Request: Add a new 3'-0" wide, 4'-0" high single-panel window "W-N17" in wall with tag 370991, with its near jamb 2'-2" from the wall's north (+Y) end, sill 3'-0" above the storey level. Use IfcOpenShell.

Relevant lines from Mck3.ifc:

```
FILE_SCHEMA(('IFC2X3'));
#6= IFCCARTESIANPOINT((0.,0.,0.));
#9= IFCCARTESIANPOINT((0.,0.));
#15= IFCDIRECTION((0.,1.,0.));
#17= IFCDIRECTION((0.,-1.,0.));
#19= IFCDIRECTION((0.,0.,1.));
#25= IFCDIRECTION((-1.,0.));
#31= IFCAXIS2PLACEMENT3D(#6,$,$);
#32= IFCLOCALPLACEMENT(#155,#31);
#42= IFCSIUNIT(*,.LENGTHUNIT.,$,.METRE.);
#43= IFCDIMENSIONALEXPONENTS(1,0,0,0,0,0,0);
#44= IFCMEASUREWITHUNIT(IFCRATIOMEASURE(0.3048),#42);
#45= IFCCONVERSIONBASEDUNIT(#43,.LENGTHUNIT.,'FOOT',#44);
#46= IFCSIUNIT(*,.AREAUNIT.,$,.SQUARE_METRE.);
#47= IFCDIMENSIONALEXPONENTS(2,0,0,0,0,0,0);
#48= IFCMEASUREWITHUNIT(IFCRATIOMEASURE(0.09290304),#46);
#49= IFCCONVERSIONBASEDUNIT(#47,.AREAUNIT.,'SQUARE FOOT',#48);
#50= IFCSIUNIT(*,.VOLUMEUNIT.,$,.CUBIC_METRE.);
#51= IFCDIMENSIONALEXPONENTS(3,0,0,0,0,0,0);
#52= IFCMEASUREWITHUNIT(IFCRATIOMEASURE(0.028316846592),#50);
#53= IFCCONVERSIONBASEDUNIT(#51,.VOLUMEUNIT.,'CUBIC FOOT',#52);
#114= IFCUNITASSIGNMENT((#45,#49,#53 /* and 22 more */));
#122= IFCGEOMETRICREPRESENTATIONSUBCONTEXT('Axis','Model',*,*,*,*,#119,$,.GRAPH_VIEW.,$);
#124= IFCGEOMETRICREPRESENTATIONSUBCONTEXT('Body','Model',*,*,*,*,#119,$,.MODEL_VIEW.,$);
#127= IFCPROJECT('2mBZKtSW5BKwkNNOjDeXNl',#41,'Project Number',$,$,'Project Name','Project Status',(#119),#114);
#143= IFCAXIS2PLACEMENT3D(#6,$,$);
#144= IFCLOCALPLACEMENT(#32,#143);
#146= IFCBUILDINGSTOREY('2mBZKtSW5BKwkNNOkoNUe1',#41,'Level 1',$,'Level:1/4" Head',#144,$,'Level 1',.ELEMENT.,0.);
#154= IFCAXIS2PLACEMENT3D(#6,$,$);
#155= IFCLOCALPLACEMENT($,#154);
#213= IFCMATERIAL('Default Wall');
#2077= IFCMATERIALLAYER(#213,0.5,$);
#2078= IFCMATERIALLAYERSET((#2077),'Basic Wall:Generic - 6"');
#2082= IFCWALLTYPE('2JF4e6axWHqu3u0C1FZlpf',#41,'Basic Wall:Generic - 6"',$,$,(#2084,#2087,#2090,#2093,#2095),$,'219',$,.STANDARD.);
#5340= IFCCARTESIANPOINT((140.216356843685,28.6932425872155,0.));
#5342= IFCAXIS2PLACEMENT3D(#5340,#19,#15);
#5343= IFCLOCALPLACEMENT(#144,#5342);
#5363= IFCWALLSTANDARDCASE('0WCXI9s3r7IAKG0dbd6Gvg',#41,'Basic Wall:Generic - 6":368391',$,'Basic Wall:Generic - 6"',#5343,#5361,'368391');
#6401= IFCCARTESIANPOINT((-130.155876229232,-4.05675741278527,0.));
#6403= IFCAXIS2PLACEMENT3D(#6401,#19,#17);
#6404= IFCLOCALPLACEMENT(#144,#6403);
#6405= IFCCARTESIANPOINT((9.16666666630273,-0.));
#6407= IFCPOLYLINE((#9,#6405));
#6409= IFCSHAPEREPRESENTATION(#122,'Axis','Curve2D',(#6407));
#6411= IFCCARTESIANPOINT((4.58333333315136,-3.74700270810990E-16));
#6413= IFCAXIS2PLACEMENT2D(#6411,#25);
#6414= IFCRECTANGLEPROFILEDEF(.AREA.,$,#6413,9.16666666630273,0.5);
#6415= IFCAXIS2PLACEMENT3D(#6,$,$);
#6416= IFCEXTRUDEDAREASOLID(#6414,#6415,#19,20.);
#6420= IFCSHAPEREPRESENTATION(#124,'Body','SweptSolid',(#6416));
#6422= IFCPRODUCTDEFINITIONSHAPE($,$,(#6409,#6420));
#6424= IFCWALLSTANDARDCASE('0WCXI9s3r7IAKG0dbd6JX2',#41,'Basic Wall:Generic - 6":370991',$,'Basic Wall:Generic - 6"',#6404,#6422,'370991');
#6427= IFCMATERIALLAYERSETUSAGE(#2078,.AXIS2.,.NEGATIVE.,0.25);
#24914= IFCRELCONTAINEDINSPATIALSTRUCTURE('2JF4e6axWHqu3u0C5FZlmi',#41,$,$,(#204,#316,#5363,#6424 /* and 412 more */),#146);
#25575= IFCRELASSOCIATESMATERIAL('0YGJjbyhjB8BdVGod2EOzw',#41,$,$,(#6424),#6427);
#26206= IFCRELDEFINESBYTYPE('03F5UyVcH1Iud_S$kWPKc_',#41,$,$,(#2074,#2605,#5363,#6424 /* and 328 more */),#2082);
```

```python
import numpy as np
import ifcopenshell
import ifcopenshell.api.feature
import ifcopenshell.api.geometry
import ifcopenshell.api.root
import ifcopenshell.api.spatial
import ifcopenshell.api.type
import ifcopenshell.geom
import ifcopenshell.util.element
import ifcopenshell.util.placement
import ifcopenshell.util.representation
import ifcopenshell.util.shape
import ifcopenshell.util.unit

model = ifcopenshell.open("Mck3.ifc")
unit_scale = ifcopenshell.util.unit.calculate_unit_scale(model)
settings = ifcopenshell.geom.settings()


def volume(element):
    """Net volume in cubic metres, openings subtracted."""
    shape = ifcopenshell.geom.create_shape(settings, element)
    return ifcopenshell.util.shape.get_volume(shape.geometry)


wall = model.by_guid("0WCXI9s3r7IAKG0dbd6JX2")
storey = ifcopenshell.util.element.get_container(wall, ifc_class="IfcBuildingStorey")
context = ifcopenshell.util.representation.get_context(model, "Model", "Body", "MODEL_VIEW")
before = volume(wall)

width, height, from_end, sill = 0.9144, 1.2192, 0.6604, 0.9144  # metres

# The wall runs along its own X axis, and the end named is its -X end.
wall_shape = ifcopenshell.geom.create_shape(settings, wall)
x, y, z = ifcopenshell.util.shape.get_vertices(wall_shape.geometry).T
start = x.min() + from_end
face, thickness = float(y.min()), float(y.max() - y.min())
wall_matrix = ifcopenshell.util.placement.get_local_placement(wall.ObjectPlacement)
level = ifcopenshell.util.placement.get_local_placement(storey.ObjectPlacement)[2, 3]


def in_wall(x, y):
    """Placement at x, y metres in the wall's axes, at sill height."""
    matrix = wall_matrix.copy()
    matrix[:, 3] = wall_matrix @ np.array([x / unit_scale, y / unit_scale, 0.0, 1.0])
    matrix[2, 3] = level + sill / unit_scale
    return matrix


# Opening: a box that overshoots both wall faces by 50 mm.
opening = ifcopenshell.api.root.create_entity(model, ifc_class="IfcOpeningElement")
box = ifcopenshell.api.geometry.add_wall_representation(
    model, context=context, length=width, height=height, thickness=thickness + 0.1
)
ifcopenshell.api.geometry.assign_representation(model, product=opening, representation=box)
ifcopenshell.api.geometry.edit_object_placement(model, product=opening, matrix=in_wall(start, face - 0.05), is_si=False)
ifcopenshell.api.feature.add_feature(model, feature=opening, element=wall)

window = ifcopenshell.api.root.create_entity(model, ifc_class="IfcWindow", name="W-N17")
window.OverallWidth, window.OverallHeight = width / unit_scale, height / unit_scale
body = ifcopenshell.api.geometry.add_window_representation(
    model,
    context=context,
    overall_width=window.OverallWidth,
    overall_height=window.OverallHeight,
    partition_type="SINGLE_PANEL",
)
ifcopenshell.api.geometry.assign_representation(model, product=window, representation=body)
ifcopenshell.api.spatial.assign_container(model, products=[window], relating_structure=storey)
fills = ifcopenshell.api.feature.add_filling(model, opening=opening, element=window)
fills.OwnerHistory = window.OwnerHistory  # required in IFC2X3

# IFC2X3 keeps the operation on the window style.
style = ifcopenshell.api.root.create_entity(model, ifc_class="IfcWindowStyle", name="W-N17")
style.OperationType, style.ConstructionType = "SINGLE_PANEL", "NOTDEFINED"
style.ParameterTakesPrecedence = style.Sizeable = False
ifcopenshell.api.type.assign_type(model, related_objects=[window], relating_type=style)

# Centre the window in the wall's thickness.
ifcopenshell.api.geometry.edit_object_placement(model, product=window, matrix=in_wall(start, face), is_si=False)
window_shape = ifcopenshell.geom.create_shape(settings, window)
depth = ifcopenshell.util.shape.get_vertices(window_shape.geometry)[:, 1]
offset = face + thickness / 2 - (depth.min() + depth.max()) / 2
ifcopenshell.api.geometry.edit_object_placement(model, product=window, matrix=in_wall(start, offset), is_si=False)

after = volume(wall)

print(f"wall volume {before:.3f} -> {after:.3f} m3")

model.write("Mck3_v2.ifc")
```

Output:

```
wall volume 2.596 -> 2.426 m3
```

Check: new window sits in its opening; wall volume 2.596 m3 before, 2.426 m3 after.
